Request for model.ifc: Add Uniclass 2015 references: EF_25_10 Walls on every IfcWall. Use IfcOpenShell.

First a look at what the model holds.

```python
import ifcopenshell

model = ifcopenshell.open("model.ifc")
print(model.schema)
print("classifications:", [c.Name for c in model.by_type("IfcClassification")])
for ifc_class in ("IfcDoor", "IfcRoof", "IfcStair", "IfcWall", "IfcWindow"):
    print(ifc_class, len(model.by_type(ifc_class)))
```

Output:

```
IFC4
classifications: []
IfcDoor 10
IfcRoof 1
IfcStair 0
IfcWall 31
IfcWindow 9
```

```python
import ifcopenshell
import ifcopenshell.api.classification

model = ifcopenshell.open("model.ifc")

system = ifcopenshell.api.classification.add_classification(model, classification="Uniclass 2015")

codes = {
    "IfcWall": ("EF_25_10", "Walls"),
}
for ifc_class, (code, name) in codes.items():
    products = model.by_type(ifc_class)
    ifcopenshell.api.classification.add_reference(
        model, products=products, classification=system, identification=code, name=name
    )
    print(code, len(products))

model.write("model_updated.ifc")
```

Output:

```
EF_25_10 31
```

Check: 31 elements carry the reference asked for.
